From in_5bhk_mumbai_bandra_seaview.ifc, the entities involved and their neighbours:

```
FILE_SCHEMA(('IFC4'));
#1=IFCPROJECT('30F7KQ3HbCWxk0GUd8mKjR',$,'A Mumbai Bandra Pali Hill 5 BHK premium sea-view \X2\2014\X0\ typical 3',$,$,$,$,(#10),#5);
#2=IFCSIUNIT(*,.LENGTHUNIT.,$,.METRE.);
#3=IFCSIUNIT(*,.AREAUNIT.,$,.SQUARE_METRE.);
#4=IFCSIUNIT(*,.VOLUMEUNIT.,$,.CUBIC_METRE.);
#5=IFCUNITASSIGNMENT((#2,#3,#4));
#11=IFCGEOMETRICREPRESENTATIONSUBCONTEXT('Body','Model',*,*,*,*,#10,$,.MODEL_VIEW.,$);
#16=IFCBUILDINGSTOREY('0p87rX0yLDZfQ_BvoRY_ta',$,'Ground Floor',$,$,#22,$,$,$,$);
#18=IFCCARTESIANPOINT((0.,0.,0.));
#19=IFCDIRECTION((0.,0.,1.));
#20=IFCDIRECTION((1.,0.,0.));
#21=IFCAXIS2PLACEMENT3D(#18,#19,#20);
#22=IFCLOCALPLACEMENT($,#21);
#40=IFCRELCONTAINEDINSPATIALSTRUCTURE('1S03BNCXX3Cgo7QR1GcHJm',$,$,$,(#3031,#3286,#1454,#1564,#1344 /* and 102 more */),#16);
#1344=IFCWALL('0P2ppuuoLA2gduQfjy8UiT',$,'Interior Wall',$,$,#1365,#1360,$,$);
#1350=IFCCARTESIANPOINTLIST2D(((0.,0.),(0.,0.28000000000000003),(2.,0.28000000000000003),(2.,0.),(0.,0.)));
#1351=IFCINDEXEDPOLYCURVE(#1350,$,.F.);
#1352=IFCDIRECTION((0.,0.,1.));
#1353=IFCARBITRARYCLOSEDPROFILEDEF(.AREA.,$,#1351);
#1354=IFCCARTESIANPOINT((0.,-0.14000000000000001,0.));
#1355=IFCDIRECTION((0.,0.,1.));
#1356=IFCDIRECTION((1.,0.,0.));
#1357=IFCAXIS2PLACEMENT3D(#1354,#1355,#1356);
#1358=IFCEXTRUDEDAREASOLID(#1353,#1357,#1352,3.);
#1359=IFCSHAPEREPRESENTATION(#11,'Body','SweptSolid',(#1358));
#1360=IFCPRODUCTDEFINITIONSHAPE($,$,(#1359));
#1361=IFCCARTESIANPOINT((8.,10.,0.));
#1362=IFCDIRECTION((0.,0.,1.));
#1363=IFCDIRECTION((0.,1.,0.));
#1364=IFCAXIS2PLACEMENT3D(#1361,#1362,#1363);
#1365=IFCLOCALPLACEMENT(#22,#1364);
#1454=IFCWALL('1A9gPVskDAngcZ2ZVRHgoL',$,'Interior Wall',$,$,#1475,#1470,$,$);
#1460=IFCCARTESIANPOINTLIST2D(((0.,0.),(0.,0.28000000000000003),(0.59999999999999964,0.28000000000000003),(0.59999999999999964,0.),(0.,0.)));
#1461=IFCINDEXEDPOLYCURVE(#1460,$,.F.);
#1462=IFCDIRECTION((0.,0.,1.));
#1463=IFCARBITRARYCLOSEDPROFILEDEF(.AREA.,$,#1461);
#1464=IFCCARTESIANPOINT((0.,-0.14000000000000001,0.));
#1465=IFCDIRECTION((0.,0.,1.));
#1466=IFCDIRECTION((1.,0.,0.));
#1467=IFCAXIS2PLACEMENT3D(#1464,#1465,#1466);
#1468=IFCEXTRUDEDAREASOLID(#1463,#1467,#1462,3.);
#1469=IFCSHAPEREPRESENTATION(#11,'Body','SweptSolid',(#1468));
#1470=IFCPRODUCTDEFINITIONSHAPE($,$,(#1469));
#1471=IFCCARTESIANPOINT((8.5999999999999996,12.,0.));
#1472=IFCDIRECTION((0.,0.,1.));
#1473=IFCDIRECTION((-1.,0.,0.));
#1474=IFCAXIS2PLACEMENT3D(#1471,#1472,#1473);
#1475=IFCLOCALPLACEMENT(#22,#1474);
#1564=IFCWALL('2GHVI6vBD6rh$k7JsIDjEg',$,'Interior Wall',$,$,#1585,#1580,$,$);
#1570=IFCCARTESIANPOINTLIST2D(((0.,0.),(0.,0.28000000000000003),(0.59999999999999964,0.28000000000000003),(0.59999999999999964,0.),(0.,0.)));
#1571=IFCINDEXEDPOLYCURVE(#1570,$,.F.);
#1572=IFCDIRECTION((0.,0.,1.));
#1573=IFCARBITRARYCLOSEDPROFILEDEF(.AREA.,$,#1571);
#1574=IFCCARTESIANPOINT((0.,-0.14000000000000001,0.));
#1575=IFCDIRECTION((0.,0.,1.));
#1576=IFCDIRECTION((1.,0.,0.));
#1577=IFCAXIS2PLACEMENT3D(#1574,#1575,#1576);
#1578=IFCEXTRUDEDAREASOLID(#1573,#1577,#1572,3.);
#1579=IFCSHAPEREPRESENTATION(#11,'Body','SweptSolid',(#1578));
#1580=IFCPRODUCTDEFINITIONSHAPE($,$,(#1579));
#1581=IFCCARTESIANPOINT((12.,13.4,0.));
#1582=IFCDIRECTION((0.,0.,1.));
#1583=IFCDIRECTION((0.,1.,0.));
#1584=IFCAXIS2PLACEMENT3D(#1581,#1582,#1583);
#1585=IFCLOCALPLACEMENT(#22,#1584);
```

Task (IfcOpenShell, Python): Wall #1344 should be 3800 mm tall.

```python
import ifcopenshell
import ifcopenshell.geom
import ifcopenshell.util.representation
import ifcopenshell.util.shape

model = ifcopenshell.open("in_5bhk_mumbai_bandra_seaview.ifc")
settings = ifcopenshell.geom.settings()


def volume(element):
    """Net volume in cubic metres, openings subtracted."""
    shape = ifcopenshell.geom.create_shape(settings, element)
    return ifcopenshell.util.shape.get_volume(shape.geometry)


wall = model.by_guid("0P2ppuuoLA2gduQfjy8UiT")
before = volume(wall)

body = ifcopenshell.util.representation.get_representation(wall, "Model", "Body")
solid = body.Items[0]
old_height = solid.Depth
solid.Depth = 3.8
after = volume(wall)

print(f"height {old_height:g} -> {solid.Depth:g}, volume {before:.3f} -> {after:.3f} m3")

model.write("in_5bhk_mumbai_bandra_seaview-out.ifc")
```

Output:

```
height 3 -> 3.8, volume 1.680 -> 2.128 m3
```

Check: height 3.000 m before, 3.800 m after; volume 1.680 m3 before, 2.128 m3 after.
